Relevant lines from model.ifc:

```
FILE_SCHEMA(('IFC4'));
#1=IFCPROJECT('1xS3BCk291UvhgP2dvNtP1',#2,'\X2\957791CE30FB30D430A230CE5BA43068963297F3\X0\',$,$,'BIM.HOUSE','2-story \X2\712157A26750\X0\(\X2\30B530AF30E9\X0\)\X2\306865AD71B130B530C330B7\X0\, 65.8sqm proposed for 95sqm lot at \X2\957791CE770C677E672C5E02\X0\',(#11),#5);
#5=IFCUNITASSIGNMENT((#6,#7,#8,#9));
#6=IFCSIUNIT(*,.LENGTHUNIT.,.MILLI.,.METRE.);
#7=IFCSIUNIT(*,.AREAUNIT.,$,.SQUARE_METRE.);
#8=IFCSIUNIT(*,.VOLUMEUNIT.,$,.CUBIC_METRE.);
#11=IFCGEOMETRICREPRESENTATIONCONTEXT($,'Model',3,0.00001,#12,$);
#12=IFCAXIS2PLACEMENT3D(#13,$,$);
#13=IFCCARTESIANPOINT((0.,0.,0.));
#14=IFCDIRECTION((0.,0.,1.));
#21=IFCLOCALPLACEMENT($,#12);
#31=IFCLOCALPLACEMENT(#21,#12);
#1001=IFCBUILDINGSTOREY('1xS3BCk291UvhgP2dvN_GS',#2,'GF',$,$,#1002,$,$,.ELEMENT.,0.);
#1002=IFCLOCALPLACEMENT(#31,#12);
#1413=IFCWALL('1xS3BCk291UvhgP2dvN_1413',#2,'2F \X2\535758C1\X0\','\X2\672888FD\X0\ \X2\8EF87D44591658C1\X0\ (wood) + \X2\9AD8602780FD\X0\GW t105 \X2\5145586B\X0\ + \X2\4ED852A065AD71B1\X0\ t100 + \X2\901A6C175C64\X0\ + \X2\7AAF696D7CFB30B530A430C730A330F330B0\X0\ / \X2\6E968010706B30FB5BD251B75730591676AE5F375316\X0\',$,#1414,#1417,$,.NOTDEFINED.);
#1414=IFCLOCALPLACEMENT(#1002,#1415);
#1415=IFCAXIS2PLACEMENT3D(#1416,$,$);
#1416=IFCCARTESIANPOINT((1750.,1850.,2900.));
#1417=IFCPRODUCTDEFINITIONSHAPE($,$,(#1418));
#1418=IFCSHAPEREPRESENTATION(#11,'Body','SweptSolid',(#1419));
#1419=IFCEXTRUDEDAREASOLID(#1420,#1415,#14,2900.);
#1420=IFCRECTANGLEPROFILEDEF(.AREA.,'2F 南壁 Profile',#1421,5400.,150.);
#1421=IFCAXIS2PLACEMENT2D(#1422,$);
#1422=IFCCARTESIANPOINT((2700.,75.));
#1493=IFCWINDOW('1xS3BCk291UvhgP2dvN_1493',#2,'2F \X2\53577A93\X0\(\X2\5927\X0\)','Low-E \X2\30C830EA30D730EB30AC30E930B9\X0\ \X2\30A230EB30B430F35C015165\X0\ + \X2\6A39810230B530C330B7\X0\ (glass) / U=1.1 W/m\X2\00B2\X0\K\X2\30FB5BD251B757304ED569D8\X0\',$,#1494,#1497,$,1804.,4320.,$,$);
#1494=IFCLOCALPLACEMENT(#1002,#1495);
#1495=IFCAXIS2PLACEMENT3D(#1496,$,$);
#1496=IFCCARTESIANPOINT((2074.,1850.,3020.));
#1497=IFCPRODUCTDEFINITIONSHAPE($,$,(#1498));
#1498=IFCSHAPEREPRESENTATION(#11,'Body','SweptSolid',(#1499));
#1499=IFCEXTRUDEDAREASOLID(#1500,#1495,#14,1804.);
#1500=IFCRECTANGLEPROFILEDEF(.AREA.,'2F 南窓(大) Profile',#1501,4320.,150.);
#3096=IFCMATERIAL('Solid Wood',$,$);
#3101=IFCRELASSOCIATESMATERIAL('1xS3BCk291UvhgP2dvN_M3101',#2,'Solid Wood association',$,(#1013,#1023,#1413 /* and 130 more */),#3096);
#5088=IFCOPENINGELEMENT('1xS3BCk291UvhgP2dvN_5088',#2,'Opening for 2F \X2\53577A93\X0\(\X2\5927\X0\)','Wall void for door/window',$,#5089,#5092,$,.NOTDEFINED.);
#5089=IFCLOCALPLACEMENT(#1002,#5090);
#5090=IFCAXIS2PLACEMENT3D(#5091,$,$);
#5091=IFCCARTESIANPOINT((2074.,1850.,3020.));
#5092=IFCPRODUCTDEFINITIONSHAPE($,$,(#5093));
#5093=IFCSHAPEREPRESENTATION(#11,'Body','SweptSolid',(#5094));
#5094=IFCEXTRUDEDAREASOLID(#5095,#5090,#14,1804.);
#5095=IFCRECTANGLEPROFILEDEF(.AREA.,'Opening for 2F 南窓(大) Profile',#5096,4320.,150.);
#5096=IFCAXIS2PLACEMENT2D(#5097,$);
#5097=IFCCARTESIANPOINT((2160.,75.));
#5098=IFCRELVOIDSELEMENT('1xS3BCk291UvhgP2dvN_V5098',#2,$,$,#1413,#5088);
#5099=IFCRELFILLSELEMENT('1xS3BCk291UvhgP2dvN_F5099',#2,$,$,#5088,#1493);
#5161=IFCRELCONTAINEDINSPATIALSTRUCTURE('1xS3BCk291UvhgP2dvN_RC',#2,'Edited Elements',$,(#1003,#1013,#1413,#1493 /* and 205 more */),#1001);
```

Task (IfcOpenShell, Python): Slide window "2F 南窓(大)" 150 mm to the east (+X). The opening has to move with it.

```python
import ifcopenshell
import ifcopenshell.api.geometry
import ifcopenshell.util.placement
import ifcopenshell.util.unit

model = ifcopenshell.open("model.ifc")
unit_scale = ifcopenshell.util.unit.calculate_unit_scale(model)

window = model.by_guid("1xS3BCk291UvhgP2dvN_1493")
opening = window.FillsVoids[0].RelatingOpeningElement
wall = opening.VoidsElements[0].RelatingBuildingElement

wall_matrix = ifcopenshell.util.placement.get_local_placement(wall.ObjectPlacement)
shift = wall_matrix[:3, 0] * 0.15 / unit_scale
before = ifcopenshell.util.placement.get_local_placement(window.ObjectPlacement)[:3, 3].copy()

# The window is not placed relative to its opening, so move both.
for product in (opening, window):
    matrix = ifcopenshell.util.placement.get_local_placement(product.ObjectPlacement)
    matrix[:3, 3] += shift
    ifcopenshell.api.geometry.edit_object_placement(model, product=product, matrix=matrix, is_si=False)

after = ifcopenshell.util.placement.get_local_placement(window.ObjectPlacement)[:3, 3]
print("window moved by", (after - before).round(3) + 0.0)

model.write("model-out.ifc")
```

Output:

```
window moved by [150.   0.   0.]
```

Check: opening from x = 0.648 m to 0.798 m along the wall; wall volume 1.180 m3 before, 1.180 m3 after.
